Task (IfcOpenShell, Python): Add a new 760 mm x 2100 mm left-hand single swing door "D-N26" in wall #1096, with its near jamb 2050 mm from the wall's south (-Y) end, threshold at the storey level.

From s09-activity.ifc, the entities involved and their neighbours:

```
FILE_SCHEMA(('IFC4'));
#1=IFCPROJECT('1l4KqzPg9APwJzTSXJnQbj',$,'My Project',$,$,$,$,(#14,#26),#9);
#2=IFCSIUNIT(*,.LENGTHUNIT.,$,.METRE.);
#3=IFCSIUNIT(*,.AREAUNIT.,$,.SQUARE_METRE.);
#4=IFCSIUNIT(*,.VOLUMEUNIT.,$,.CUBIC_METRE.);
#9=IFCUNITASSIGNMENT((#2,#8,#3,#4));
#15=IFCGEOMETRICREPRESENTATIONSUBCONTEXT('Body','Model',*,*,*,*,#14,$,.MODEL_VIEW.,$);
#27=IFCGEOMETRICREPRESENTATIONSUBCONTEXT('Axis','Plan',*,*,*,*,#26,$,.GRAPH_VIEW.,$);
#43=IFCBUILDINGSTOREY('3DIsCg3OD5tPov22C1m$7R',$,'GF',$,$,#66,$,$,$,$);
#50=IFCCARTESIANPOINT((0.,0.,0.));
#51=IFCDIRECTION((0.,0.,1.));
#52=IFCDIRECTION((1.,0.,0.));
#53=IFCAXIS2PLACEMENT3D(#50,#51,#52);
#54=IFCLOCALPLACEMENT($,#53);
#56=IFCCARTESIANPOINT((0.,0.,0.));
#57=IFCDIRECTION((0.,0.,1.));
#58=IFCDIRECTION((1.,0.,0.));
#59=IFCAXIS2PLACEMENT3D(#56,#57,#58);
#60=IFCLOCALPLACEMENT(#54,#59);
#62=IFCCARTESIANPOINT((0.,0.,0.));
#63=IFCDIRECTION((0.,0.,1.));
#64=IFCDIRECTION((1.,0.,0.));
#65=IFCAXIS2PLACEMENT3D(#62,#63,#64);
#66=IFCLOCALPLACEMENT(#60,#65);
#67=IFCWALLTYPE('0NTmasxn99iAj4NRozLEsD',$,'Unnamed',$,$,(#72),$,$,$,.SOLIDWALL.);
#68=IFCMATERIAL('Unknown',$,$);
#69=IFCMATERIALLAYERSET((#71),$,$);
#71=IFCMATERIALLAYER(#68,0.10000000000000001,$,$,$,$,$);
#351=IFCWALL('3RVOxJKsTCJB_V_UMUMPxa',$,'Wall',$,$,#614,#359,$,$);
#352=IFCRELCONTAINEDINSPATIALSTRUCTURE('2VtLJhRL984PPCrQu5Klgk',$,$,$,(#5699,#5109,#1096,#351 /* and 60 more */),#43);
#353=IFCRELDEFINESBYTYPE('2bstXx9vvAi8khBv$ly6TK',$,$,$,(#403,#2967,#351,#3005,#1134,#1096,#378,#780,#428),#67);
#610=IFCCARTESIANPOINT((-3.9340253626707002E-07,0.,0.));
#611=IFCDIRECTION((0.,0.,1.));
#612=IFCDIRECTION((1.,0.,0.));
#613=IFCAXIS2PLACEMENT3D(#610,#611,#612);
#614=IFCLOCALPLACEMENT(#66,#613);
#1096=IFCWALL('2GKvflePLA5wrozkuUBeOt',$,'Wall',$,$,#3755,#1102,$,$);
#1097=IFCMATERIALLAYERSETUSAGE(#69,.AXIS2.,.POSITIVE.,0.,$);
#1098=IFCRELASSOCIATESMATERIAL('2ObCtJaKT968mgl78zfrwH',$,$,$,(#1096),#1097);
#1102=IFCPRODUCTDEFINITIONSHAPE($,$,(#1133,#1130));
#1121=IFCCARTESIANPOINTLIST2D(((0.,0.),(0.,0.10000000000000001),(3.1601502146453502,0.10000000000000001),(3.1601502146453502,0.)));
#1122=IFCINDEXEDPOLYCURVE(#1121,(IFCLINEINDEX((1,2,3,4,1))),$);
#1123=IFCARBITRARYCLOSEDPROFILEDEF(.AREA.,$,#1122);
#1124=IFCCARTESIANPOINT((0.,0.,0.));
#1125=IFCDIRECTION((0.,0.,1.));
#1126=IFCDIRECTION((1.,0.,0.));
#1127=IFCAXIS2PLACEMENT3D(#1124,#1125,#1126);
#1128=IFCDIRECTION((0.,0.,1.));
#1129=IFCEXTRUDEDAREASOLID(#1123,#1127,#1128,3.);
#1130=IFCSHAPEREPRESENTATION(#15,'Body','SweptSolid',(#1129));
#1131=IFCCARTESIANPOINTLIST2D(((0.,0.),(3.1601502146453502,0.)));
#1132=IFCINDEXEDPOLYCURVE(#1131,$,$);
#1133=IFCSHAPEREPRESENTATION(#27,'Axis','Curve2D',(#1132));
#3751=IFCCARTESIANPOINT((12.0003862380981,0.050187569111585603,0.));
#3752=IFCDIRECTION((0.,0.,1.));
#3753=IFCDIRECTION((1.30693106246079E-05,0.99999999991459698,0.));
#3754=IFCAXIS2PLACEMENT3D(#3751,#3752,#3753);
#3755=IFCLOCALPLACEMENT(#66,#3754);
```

```python
import numpy as np
import ifcopenshell
import ifcopenshell.api.feature
import ifcopenshell.api.geometry
import ifcopenshell.api.root
import ifcopenshell.api.spatial
import ifcopenshell.geom
import ifcopenshell.util.element
import ifcopenshell.util.placement
import ifcopenshell.util.representation
import ifcopenshell.util.shape
import ifcopenshell.util.unit

model = ifcopenshell.open("s09-activity.ifc")
unit_scale = ifcopenshell.util.unit.calculate_unit_scale(model)
settings = ifcopenshell.geom.settings()


def volume(element):
    """Net volume in cubic metres, openings subtracted."""
    shape = ifcopenshell.geom.create_shape(settings, element)
    return ifcopenshell.util.shape.get_volume(shape.geometry)


wall = model.by_guid("2GKvflePLA5wrozkuUBeOt")
storey = ifcopenshell.util.element.get_container(wall, ifc_class="IfcBuildingStorey")
context = ifcopenshell.util.representation.get_context(model, "Model", "Body", "MODEL_VIEW")
before = volume(wall)

width, height, from_end, sill = 0.76, 2.1, 2.05, 0.0  # metres

# The wall runs along its own X axis, and the end named is its -X end.
wall_shape = ifcopenshell.geom.create_shape(settings, wall)
x, y, z = ifcopenshell.util.shape.get_vertices(wall_shape.geometry).T
start = x.min() + from_end
face, thickness = float(y.min()), float(y.max() - y.min())
wall_matrix = ifcopenshell.util.placement.get_local_placement(wall.ObjectPlacement)
level = ifcopenshell.util.placement.get_local_placement(storey.ObjectPlacement)[2, 3]


def in_wall(x, y):
    """Placement at x, y metres in the wall's axes, at sill height."""
    matrix = wall_matrix.copy()
    matrix[:, 3] = wall_matrix @ np.array([x / unit_scale, y / unit_scale, 0.0, 1.0])
    matrix[2, 3] = level + sill / unit_scale
    return matrix


# Opening: a box that overshoots both wall faces by 50 mm.
opening = ifcopenshell.api.root.create_entity(model, ifc_class="IfcOpeningElement", predefined_type="OPENING")
box = ifcopenshell.api.geometry.add_wall_representation(
    model, context=context, length=width, height=height, thickness=thickness + 0.1
)
ifcopenshell.api.geometry.assign_representation(model, product=opening, representation=box)
ifcopenshell.api.geometry.edit_object_placement(model, product=opening, matrix=in_wall(start, face - 0.05), is_si=False)
ifcopenshell.api.feature.add_feature(model, feature=opening, element=wall)

door = ifcopenshell.api.root.create_entity(model, ifc_class="IfcDoor", name="D-N26", predefined_type="DOOR")
door.OverallWidth, door.OverallHeight = width / unit_scale, height / unit_scale
door.OperationType = "SINGLE_SWING_LEFT"
body = ifcopenshell.api.geometry.add_door_representation(
    model,
    context=context,
    overall_width=door.OverallWidth,
    overall_height=door.OverallHeight,
    operation_type="SINGLE_SWING_LEFT",
    lining_properties={"LiningDepth": thickness / unit_scale, "ThresholdDepth": thickness / unit_scale},
)
ifcopenshell.api.geometry.assign_representation(model, product=door, representation=body)
ifcopenshell.api.spatial.assign_container(model, products=[door], relating_structure=storey)
ifcopenshell.api.feature.add_filling(model, opening=opening, element=door)

# The lining spans the wall, so the door starts at the wall face.
ifcopenshell.api.geometry.edit_object_placement(model, product=door, matrix=in_wall(start, face), is_si=False)

after = volume(wall)

print(f"wall volume {before:.3f} -> {after:.3f} m3")

model.write("s09-activity_edited.ifc")
```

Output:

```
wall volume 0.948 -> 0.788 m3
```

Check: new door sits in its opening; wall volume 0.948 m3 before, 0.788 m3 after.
